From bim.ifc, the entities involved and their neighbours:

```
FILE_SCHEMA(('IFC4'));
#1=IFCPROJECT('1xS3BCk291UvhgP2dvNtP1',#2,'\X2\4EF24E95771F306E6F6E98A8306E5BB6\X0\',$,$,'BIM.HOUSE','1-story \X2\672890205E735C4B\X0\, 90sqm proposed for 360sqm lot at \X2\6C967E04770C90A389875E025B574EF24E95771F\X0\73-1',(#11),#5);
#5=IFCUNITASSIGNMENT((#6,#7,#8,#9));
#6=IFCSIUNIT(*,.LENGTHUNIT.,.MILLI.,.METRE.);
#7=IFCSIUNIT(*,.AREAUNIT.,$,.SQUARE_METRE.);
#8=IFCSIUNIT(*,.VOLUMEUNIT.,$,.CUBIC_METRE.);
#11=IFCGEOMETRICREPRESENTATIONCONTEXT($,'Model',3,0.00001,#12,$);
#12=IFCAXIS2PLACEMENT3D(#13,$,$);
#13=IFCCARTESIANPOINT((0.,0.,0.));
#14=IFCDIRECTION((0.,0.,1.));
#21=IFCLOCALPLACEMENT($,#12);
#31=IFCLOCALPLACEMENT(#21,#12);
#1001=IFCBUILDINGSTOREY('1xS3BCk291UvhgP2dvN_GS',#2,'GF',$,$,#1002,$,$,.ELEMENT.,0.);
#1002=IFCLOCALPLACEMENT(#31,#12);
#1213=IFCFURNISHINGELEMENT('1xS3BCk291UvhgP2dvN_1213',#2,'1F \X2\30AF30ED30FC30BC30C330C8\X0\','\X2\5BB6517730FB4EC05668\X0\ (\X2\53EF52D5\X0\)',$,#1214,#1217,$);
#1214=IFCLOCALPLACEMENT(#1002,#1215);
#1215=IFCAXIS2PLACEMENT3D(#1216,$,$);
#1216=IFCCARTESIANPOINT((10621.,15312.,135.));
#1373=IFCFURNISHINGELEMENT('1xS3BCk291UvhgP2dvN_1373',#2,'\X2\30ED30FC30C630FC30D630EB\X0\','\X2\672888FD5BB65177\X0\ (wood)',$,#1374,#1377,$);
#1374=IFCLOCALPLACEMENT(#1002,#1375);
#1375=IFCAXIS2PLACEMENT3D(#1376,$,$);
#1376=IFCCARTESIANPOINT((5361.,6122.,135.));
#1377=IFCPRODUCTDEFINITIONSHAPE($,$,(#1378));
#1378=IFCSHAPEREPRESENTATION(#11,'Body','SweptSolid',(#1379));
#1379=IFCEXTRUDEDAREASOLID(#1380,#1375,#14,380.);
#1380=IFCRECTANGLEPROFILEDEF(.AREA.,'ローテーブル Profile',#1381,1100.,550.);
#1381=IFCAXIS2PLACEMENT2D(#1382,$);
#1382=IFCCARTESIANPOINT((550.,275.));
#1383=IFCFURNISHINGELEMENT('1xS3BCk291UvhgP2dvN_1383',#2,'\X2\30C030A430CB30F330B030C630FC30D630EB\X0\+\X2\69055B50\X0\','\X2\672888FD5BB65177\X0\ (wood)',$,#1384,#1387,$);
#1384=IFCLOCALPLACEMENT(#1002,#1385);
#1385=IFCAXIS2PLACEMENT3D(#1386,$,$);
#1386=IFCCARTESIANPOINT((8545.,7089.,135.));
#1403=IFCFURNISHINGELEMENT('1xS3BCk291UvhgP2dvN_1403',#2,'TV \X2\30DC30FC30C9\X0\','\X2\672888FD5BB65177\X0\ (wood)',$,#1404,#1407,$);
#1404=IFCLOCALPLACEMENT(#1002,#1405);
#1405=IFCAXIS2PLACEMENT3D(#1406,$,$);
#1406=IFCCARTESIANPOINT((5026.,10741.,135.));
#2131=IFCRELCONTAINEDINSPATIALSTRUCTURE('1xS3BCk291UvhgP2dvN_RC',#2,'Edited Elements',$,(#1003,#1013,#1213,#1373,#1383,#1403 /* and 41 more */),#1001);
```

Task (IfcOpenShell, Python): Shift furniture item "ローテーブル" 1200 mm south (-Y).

```python
import ifcopenshell
import ifcopenshell.api.geometry
import ifcopenshell.util.placement
import ifcopenshell.util.unit

model = ifcopenshell.open("bim.ifc")
unit_scale = ifcopenshell.util.unit.calculate_unit_scale(model)

item = model.by_id(1373)
matrix = ifcopenshell.util.placement.get_local_placement(item.ObjectPlacement)
matrix[1, 3] -= 1.2 / unit_scale
ifcopenshell.api.geometry.edit_object_placement(model, product=item, matrix=matrix, is_si=False)

print(ifcopenshell.util.placement.get_local_placement(item.ObjectPlacement).round(3) + 0.0)

model.write("bim_edited.ifc")
```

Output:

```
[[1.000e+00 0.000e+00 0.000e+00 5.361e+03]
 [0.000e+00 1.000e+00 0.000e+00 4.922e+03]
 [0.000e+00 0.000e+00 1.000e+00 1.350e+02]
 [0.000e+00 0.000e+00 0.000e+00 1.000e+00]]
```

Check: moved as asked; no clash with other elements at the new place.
